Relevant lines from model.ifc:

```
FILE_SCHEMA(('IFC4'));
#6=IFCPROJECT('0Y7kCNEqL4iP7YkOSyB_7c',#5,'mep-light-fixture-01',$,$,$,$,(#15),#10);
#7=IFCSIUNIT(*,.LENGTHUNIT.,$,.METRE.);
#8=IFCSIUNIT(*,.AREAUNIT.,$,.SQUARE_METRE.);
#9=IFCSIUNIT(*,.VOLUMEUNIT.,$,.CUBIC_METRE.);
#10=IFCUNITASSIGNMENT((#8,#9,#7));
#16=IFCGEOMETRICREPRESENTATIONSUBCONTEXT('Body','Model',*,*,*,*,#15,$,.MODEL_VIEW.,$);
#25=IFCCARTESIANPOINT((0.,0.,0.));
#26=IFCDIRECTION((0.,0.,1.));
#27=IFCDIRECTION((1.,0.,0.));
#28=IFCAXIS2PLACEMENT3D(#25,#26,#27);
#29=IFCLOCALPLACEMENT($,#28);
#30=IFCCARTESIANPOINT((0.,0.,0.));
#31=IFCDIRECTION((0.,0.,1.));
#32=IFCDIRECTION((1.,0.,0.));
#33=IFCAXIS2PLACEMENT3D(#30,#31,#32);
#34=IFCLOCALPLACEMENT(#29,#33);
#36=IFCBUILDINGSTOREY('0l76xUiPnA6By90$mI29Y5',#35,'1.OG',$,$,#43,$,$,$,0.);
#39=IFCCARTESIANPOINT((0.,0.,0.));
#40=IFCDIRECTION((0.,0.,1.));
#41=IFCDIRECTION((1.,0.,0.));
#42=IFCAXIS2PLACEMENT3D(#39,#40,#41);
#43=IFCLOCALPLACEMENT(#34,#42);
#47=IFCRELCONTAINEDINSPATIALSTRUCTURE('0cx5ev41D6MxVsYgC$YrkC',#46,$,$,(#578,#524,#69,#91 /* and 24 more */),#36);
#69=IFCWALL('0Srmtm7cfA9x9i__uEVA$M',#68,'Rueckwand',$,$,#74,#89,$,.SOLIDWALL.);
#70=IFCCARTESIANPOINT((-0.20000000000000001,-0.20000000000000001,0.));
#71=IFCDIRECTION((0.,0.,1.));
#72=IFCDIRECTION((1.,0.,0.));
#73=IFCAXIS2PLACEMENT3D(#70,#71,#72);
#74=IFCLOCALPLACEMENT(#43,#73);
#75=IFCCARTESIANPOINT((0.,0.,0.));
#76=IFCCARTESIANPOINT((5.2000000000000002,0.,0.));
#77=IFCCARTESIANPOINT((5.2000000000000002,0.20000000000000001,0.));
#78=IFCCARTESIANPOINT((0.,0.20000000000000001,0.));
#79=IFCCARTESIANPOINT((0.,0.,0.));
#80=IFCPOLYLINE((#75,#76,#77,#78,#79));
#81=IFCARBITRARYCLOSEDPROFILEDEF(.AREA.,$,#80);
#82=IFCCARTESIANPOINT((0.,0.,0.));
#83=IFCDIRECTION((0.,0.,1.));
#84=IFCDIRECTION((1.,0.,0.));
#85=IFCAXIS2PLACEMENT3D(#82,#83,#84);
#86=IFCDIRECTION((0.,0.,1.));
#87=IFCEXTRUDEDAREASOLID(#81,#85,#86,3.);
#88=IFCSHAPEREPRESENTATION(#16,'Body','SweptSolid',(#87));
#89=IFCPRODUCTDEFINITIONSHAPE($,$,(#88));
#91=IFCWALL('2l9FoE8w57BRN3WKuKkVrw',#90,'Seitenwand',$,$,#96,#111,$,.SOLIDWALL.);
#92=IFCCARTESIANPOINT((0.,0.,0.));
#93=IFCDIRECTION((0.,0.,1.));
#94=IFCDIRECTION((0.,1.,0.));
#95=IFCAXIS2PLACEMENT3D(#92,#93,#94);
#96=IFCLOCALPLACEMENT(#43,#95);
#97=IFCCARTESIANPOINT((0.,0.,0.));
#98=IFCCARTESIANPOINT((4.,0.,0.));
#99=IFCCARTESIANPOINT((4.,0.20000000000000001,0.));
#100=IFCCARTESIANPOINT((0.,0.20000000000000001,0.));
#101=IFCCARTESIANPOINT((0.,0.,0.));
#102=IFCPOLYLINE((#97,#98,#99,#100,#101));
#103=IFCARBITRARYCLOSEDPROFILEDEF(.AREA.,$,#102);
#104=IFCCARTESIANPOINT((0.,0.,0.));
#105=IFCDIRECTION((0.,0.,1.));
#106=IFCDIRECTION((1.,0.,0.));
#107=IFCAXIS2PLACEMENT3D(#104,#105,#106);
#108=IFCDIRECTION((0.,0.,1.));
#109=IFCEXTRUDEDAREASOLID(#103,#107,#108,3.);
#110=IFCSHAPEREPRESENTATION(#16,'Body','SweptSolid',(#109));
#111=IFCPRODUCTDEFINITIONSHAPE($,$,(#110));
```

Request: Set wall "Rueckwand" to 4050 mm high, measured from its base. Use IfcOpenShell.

```python
import ifcopenshell
import ifcopenshell.geom
import ifcopenshell.util.representation
import ifcopenshell.util.shape

model = ifcopenshell.open("model.ifc")
settings = ifcopenshell.geom.settings()


def volume(element):
    """Net volume in cubic metres, openings subtracted."""
    shape = ifcopenshell.geom.create_shape(settings, element)
    return ifcopenshell.util.shape.get_volume(shape.geometry)


wall = model.by_guid("0Srmtm7cfA9x9i__uEVA$M")
before = volume(wall)

body = ifcopenshell.util.representation.get_representation(wall, "Model", "Body")
solid = body.Items[0]
old_height = solid.Depth
solid.Depth = 4.05
after = volume(wall)

print(f"height {old_height:g} -> {solid.Depth:g}, volume {before:.3f} -> {after:.3f} m3")

model.write("model_updated.ifc")
```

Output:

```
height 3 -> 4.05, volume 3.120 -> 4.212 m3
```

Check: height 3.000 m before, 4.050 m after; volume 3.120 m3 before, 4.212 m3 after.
